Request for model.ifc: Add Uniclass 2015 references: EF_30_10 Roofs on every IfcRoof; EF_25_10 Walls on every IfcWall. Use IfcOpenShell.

First a look at what the model holds.

```python
import ifcopenshell

model = ifcopenshell.open("model.ifc")
print(model.schema)
print("classifications:", [c.Name for c in model.by_type("IfcClassification")])
for ifc_class in ("IfcDoor", "IfcRoof", "IfcStair", "IfcWall", "IfcWindow"):
    print(ifc_class, len(model.by_type(ifc_class)))
```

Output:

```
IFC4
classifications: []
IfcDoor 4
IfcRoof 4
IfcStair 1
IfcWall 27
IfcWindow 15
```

```python
import ifcopenshell
import ifcopenshell.api.classification

model = ifcopenshell.open("model.ifc")

system = ifcopenshell.api.classification.add_classification(model, classification="Uniclass 2015")

codes = {
    "IfcRoof": ("EF_30_10", "Roofs"),
    "IfcWall": ("EF_25_10", "Walls"),
}
for ifc_class, (code, name) in codes.items():
    products = model.by_type(ifc_class)
    ifcopenshell.api.classification.add_reference(
        model, products=products, classification=system, identification=code, name=name
    )
    print(code, len(products))

model.write("model_v2.ifc")
```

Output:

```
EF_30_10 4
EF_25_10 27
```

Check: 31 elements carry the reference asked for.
